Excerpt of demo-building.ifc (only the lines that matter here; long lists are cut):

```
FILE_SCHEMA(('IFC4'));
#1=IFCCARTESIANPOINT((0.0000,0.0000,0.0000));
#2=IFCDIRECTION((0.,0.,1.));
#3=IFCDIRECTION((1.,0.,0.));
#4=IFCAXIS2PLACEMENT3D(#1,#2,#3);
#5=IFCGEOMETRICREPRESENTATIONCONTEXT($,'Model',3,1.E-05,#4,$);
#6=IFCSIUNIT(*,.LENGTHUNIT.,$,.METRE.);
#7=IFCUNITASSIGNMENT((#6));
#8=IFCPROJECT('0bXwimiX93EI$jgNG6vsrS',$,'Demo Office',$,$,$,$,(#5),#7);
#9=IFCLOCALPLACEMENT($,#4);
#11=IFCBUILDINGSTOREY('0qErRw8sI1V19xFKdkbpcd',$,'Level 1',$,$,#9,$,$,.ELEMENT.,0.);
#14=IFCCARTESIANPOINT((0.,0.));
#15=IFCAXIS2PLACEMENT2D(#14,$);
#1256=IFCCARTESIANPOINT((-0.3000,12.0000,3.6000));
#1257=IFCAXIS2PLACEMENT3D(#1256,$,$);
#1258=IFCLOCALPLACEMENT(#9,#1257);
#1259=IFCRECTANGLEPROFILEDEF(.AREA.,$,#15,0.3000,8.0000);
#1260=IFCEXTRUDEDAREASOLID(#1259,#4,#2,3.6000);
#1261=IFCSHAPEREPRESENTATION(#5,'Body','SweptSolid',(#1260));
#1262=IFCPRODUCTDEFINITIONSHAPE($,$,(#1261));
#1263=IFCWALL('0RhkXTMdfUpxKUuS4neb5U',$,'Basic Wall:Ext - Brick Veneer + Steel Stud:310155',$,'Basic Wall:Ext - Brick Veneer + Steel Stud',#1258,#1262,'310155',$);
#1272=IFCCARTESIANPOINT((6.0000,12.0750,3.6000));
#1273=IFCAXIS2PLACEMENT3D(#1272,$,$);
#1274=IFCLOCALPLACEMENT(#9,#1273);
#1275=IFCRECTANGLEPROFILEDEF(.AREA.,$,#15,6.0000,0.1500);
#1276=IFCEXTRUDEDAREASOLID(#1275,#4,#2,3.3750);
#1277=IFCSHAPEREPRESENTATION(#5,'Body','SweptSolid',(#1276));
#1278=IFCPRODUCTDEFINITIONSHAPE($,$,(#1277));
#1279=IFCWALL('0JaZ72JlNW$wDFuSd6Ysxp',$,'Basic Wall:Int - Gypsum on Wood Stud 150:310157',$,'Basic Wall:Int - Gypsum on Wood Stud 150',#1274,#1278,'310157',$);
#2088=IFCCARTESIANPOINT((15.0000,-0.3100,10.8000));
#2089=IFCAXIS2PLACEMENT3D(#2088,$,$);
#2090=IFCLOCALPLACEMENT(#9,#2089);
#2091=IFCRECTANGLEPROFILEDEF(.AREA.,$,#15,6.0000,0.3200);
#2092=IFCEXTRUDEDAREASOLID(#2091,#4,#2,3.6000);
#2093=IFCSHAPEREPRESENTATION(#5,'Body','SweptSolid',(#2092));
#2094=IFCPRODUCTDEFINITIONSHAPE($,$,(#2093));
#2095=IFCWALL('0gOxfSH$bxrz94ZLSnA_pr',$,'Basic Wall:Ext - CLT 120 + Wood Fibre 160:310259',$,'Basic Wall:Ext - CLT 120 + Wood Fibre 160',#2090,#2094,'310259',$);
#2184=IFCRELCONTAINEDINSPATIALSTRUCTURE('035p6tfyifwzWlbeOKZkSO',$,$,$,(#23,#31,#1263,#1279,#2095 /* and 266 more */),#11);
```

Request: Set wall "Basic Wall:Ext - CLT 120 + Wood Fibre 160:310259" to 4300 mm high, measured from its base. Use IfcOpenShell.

```python
import ifcopenshell
import ifcopenshell.geom
import ifcopenshell.util.shape
import ifcopenshell.util.unit

model = ifcopenshell.open("demo-building.ifc")
unit_scale = ifcopenshell.util.unit.calculate_unit_scale(model)
settings = ifcopenshell.geom.settings()


def volume(element):
    """Net volume in cubic metres, openings subtracted."""
    shape = ifcopenshell.geom.create_shape(settings, element)
    return ifcopenshell.util.shape.get_volume(shape.geometry)


wall = model.by_id(2095)
before = volume(wall)

body = next(r for r in wall.Representation.Representations if r.RepresentationIdentifier == "Body")
solid = body.Items[0]
old_height = solid.Depth
solid.Depth = 4.3 / unit_scale
after = volume(wall)

print(f"height {old_height:g} -> {solid.Depth:g}, volume {before:.3f} -> {after:.3f} m3")

model.write("demo-building_v2.ifc")
```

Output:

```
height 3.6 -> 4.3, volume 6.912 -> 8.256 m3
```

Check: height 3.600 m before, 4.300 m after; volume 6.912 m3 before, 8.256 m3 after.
